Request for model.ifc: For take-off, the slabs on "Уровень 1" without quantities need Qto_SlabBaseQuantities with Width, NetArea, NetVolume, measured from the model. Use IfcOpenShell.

First a look at what the model holds.

```python
import ifcopenshell
import ifcopenshell.util.element
import ifcopenshell.util.unit

model = ifcopenshell.open("model.ifc")
print(model.schema)
for unit_type in ("LENGTHUNIT", "AREAUNIT", "VOLUMEUNIT"):
    print(unit_type, ifcopenshell.util.unit.calculate_unit_scale(model, unit_type))
storey = next(s for s in model.by_type("IfcBuildingStorey") if s.Name == "Уровень 1")
slabs = [e for e in ifcopenshell.util.element.get_decomposition(storey) if e.is_a("IfcSlab")]
for e in sorted(slabs, key=lambda e: e.id()):
    print(e.id(), e.is_a(), e.Name, list(ifcopenshell.util.element.get_psets(e, qtos_only=True)), sep=" | ")
```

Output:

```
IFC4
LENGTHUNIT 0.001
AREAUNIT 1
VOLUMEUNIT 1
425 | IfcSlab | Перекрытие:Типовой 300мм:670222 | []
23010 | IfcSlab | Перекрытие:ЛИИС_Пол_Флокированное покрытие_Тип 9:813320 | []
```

```python
import ifcopenshell
import ifcopenshell.api.pset
import ifcopenshell.geom
import ifcopenshell.util.element
import ifcopenshell.util.shape
import ifcopenshell.util.unit

model = ifcopenshell.open("model.ifc")
unit_scale = ifcopenshell.util.unit.calculate_unit_scale(model)
area_scale = ifcopenshell.util.unit.calculate_unit_scale(model, "AREAUNIT")
volume_scale = ifcopenshell.util.unit.calculate_unit_scale(model, "VOLUMEUNIT")
settings = ifcopenshell.geom.settings()

storey = next(s for s in model.by_type("IfcBuildingStorey") if s.Name == "Уровень 1")
slabs = [e for e in ifcopenshell.util.element.get_decomposition(storey) if e.is_a("IfcSlab")]

for e in sorted(slabs, key=lambda e: e.id()):
    if ifcopenshell.util.element.get_psets(e, qtos_only=True, should_inherit=False):
        continue
    # Geometry comes back in metres, in the element's own axes.
    shape = ifcopenshell.geom.create_shape(settings, e)
    values = {
        "Width": ifcopenshell.util.shape.get_z(shape.geometry) / unit_scale,
        "NetArea": ifcopenshell.util.shape.get_footprint_area(shape.geometry) / area_scale,
        "NetVolume": ifcopenshell.util.shape.get_volume(shape.geometry) / volume_scale,
    }
    qto = ifcopenshell.api.pset.add_qto(model, product=e, name="Qto_SlabBaseQuantities")
    ifcopenshell.api.pset.edit_qto(model, qto=qto, properties=values)
    print(e.id(), {k: round(v, 3) for k, v in values.items()})

model.write("model_rev.ifc")
```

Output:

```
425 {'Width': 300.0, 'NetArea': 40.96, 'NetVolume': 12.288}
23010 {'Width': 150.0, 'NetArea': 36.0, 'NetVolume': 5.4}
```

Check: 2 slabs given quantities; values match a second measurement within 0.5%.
